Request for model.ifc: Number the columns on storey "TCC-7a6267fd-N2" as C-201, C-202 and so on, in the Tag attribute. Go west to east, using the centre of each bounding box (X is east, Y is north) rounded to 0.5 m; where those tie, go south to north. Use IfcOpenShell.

First a look at what the model holds.

```python
import ifcopenshell
import ifcopenshell.util.element
import ifcopenshell.util.placement

model = ifcopenshell.open("model.ifc")
print(model.schema)
storey = next(s for s in model.by_type("IfcBuildingStorey") if s.Name == "TCC-7a6267fd-N2")
columns = [e for e in ifcopenshell.util.element.get_decomposition(storey) if e.is_a("IfcColumn")]
for e in sorted(columns, key=lambda e: e.id()):
    origin = ifcopenshell.util.placement.get_local_placement(e.ObjectPlacement)[:3, 3]
    print(e.id(), e.Tag, e.Name, origin.round(2) + 0.0, sep=" | ")
```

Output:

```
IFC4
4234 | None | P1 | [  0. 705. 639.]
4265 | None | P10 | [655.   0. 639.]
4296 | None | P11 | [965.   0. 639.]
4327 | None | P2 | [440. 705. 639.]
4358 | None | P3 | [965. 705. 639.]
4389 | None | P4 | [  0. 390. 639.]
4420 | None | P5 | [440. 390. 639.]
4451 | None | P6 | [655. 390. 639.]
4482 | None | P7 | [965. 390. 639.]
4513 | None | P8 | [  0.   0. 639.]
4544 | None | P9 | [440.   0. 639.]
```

```python
import ifcopenshell
import ifcopenshell.geom
import ifcopenshell.util.element
import ifcopenshell.util.shape

model = ifcopenshell.open("model.ifc")
settings = ifcopenshell.geom.settings()
settings.set("use-world-coords", True)


def centre(element):
    shape = ifcopenshell.geom.create_shape(settings, element)
    return ifcopenshell.util.shape.get_bbox_centroid(shape.geometry)


storey = next(s for s in model.by_type("IfcBuildingStorey") if s.Name == "TCC-7a6267fd-N2")
columns = [e for e in ifcopenshell.util.element.get_decomposition(storey) if e.is_a("IfcColumn")]

# Insertion points can sit at a corner or the storey origin, so sort by the geometry (in metres).
centres = {e: centre(e) for e in columns}
columns.sort(key=lambda e: (round(centres[e][0] / 0.5), centres[e][1]))

for i, e in enumerate(columns, start=1):
    number = f"C-2{i:02d}"
    e.Tag = number
    print(e.id(), number)

model.write("model_rev.ifc")
```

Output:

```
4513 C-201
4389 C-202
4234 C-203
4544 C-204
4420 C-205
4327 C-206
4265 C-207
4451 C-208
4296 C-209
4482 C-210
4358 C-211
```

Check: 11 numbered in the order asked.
